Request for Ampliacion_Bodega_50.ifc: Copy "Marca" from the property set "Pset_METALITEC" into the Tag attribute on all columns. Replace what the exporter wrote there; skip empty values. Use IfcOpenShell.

First a look at what the model holds.

```python
import ifcopenshell
import ifcopenshell.util.element

model = ifcopenshell.open("Ampliacion_Bodega_50.ifc")
print(model.schema)
columns = model.by_type("IfcColumn")
print(len(columns), "columns")
for e in columns[:8]:
    source = ifcopenshell.util.element.get_pset(e, "Pset_METALITEC", "Marca")
    target = e.Tag
    print(e.id(), repr(source), repr(target), sep=" | ")
```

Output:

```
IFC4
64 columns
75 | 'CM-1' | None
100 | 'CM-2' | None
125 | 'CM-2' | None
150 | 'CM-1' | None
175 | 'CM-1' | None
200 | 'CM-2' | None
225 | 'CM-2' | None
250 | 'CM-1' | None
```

```python
import ifcopenshell
import ifcopenshell.util.element

model = ifcopenshell.open("Ampliacion_Bodega_50.ifc")

count = 0
for e in model.by_type("IfcColumn"):
    value = ifcopenshell.util.element.get_pset(e, "Pset_METALITEC", "Marca")
    current = e.Tag
    if not value or not value.strip() or current == value:
        continue
    e.Tag = value
    count += 1

print(count, "columns updated")

model.write("Ampliacion_Bodega_50_updated.ifc")
```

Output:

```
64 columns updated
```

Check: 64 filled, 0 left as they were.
